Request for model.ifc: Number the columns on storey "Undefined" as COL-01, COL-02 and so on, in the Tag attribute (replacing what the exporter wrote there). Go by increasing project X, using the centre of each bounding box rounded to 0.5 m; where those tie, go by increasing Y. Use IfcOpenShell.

First a look at what the model holds.

```python
import ifcopenshell
import ifcopenshell.util.element
import ifcopenshell.util.placement

model = ifcopenshell.open("model.ifc")
print(model.schema)
storey = next(s for s in model.by_type("IfcBuildingStorey") if s.Name == "Undefined")
columns = [e for e in ifcopenshell.util.element.get_decomposition(storey) if e.is_a("IfcColumn")]
for e in sorted(columns, key=lambda e: e.id()):
    origin = ifcopenshell.util.placement.get_local_placement(e.ObjectPlacement)[:3, 3]
    print(e.id(), e.Tag, e.Name, origin.round(2) + 0.0, sep=" | ")
```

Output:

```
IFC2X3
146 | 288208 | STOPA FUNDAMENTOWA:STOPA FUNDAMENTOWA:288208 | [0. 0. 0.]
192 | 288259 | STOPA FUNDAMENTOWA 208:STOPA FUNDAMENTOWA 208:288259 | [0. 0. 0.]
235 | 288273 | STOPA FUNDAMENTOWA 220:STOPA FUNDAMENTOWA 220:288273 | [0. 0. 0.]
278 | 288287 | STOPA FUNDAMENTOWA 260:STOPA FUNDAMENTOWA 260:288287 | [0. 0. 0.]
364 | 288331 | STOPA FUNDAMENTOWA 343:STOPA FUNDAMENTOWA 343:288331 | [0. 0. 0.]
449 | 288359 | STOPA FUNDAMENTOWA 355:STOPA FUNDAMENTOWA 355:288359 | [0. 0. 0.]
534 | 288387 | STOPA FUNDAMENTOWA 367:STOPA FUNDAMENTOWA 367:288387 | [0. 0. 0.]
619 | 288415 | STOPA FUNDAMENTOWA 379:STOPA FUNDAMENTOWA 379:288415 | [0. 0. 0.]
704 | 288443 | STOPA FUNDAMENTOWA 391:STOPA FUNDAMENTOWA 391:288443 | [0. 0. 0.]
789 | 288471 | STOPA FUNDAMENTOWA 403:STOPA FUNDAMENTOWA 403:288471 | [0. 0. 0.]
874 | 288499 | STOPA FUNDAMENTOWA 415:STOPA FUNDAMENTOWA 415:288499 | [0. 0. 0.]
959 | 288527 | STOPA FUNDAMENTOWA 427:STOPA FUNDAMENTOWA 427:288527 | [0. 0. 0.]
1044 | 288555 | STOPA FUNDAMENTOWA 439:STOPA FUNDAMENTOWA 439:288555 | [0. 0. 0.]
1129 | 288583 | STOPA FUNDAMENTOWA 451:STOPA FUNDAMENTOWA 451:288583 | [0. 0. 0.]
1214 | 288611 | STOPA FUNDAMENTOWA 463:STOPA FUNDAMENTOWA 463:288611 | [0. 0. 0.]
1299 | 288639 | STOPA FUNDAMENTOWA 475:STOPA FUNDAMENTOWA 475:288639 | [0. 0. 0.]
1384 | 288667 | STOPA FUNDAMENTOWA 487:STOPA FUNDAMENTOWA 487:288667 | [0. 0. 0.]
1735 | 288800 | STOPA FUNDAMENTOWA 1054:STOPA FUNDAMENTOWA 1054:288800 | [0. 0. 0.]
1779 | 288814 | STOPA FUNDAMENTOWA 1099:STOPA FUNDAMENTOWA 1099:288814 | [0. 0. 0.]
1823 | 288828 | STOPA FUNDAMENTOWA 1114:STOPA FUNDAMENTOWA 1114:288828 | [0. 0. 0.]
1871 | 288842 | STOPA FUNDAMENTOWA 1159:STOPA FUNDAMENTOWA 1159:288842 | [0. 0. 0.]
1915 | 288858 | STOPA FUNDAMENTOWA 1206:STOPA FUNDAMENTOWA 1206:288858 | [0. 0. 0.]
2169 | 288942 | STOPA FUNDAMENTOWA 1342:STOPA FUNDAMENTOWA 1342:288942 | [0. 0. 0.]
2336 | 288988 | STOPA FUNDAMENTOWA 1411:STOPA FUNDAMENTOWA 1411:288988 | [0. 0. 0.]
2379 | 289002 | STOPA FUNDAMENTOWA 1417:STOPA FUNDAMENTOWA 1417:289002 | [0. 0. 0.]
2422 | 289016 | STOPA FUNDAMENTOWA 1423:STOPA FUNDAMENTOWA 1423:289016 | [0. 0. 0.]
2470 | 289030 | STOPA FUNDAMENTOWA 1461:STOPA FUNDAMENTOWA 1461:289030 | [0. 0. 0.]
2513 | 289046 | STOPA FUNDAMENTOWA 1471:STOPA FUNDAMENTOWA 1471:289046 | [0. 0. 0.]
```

```python
import ifcopenshell
import ifcopenshell.geom
import ifcopenshell.util.element
import ifcopenshell.util.shape

model = ifcopenshell.open("model.ifc")
settings = ifcopenshell.geom.settings()
settings.set("use-world-coords", True)


def centre(element):
    shape = ifcopenshell.geom.create_shape(settings, element)
    return ifcopenshell.util.shape.get_bbox_centroid(shape.geometry)


storey = next(s for s in model.by_type("IfcBuildingStorey") if s.Name == "Undefined")
columns = [e for e in ifcopenshell.util.element.get_decomposition(storey) if e.is_a("IfcColumn")]

# Insertion points can sit at a corner or the storey origin, so sort by the geometry (in metres).
centres = {e: centre(e) for e in columns}
columns.sort(key=lambda e: (round(centres[e][0] / 0.5), centres[e][1]))

for i, e in enumerate(columns, start=1):
    number = f"COL-{i:02d}"
    e.Tag = number
    print(e.id(), number)

model.write("model_edited.ifc")
```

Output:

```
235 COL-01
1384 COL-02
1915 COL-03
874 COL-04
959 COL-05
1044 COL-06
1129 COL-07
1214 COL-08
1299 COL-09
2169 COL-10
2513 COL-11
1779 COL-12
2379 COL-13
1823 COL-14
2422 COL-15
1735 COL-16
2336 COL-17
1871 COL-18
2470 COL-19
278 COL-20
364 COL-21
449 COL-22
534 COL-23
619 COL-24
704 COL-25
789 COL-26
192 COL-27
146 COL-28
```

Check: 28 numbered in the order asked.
